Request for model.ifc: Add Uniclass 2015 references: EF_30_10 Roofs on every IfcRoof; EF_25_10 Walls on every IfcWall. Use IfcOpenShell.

First a look at what the model holds.

```python
import ifcopenshell

model = ifcopenshell.open("model.ifc")
print(model.schema)
print("classifications:", [c.Name for c in model.by_type("IfcClassification")])
for ifc_class in ("IfcDoor", "IfcRoof", "IfcStair", "IfcWall", "IfcWindow"):
    print(ifc_class, len(model.by_type(ifc_class)))
```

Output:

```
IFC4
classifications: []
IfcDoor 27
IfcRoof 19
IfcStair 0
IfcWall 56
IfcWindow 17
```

```python
import ifcopenshell
import ifcopenshell.api.classification

model = ifcopenshell.open("model.ifc")

system = ifcopenshell.api.classification.add_classification(model, classification="Uniclass 2015")

codes = {
    "IfcRoof": ("EF_30_10", "Roofs"),
    "IfcWall": ("EF_25_10", "Walls"),
}
for ifc_class, (code, name) in codes.items():
    products = model.by_type(ifc_class)
    ifcopenshell.api.classification.add_reference(
        model, products=products, classification=system, identification=code, name=name
    )
    print(code, len(products))

model.write("model-out.ifc")
```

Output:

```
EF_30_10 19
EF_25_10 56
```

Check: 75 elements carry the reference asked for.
